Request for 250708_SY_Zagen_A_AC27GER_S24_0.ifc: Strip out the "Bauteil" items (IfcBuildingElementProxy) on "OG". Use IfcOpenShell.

First a look at what the model holds.

```python
import ifcopenshell
import ifcopenshell.util.element

model = ifcopenshell.open("250708_SY_Zagen_A_AC27GER_S24_0.ifc")
print(model.schema)
storey = next(s for s in model.by_type("IfcBuildingStorey") if s.Name == "OG")
proxies = [e for e in ifcopenshell.util.element.get_decomposition(storey) if e.is_a("IfcBuildingElementProxy")]
seen = {}
for e in proxies:
    element_type = ifcopenshell.util.element.get_type(e)
    name = element_type.Name if element_type not in (None, e) else None
    seen[name] = seen.get(name, 0) + 1
for name, count in sorted(seen.items(), key=str):
    print(count, "x", name)
```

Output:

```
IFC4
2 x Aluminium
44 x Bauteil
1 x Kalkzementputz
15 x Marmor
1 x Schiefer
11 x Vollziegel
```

```python
import ifcopenshell
import ifcopenshell.api.root
import ifcopenshell.util.element

model = ifcopenshell.open("250708_SY_Zagen_A_AC27GER_S24_0.ifc")

storey = next(s for s in model.by_type("IfcBuildingStorey") if s.Name == "OG")
proxies = [e for e in ifcopenshell.util.element.get_decomposition(storey) if e.is_a("IfcBuildingElementProxy")]
targets = [e for e in proxies if (t := ifcopenshell.util.element.get_type(e)) not in (None, e) and t.Name == "Bauteil"]

for e in targets:
    ifcopenshell.api.root.remove_product(model, product=e)
print(len(targets), "removed")

model.write("250708_SY_Zagen_A_AC27GER_S24_0_v2.ifc")
```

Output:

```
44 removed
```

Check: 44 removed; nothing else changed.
